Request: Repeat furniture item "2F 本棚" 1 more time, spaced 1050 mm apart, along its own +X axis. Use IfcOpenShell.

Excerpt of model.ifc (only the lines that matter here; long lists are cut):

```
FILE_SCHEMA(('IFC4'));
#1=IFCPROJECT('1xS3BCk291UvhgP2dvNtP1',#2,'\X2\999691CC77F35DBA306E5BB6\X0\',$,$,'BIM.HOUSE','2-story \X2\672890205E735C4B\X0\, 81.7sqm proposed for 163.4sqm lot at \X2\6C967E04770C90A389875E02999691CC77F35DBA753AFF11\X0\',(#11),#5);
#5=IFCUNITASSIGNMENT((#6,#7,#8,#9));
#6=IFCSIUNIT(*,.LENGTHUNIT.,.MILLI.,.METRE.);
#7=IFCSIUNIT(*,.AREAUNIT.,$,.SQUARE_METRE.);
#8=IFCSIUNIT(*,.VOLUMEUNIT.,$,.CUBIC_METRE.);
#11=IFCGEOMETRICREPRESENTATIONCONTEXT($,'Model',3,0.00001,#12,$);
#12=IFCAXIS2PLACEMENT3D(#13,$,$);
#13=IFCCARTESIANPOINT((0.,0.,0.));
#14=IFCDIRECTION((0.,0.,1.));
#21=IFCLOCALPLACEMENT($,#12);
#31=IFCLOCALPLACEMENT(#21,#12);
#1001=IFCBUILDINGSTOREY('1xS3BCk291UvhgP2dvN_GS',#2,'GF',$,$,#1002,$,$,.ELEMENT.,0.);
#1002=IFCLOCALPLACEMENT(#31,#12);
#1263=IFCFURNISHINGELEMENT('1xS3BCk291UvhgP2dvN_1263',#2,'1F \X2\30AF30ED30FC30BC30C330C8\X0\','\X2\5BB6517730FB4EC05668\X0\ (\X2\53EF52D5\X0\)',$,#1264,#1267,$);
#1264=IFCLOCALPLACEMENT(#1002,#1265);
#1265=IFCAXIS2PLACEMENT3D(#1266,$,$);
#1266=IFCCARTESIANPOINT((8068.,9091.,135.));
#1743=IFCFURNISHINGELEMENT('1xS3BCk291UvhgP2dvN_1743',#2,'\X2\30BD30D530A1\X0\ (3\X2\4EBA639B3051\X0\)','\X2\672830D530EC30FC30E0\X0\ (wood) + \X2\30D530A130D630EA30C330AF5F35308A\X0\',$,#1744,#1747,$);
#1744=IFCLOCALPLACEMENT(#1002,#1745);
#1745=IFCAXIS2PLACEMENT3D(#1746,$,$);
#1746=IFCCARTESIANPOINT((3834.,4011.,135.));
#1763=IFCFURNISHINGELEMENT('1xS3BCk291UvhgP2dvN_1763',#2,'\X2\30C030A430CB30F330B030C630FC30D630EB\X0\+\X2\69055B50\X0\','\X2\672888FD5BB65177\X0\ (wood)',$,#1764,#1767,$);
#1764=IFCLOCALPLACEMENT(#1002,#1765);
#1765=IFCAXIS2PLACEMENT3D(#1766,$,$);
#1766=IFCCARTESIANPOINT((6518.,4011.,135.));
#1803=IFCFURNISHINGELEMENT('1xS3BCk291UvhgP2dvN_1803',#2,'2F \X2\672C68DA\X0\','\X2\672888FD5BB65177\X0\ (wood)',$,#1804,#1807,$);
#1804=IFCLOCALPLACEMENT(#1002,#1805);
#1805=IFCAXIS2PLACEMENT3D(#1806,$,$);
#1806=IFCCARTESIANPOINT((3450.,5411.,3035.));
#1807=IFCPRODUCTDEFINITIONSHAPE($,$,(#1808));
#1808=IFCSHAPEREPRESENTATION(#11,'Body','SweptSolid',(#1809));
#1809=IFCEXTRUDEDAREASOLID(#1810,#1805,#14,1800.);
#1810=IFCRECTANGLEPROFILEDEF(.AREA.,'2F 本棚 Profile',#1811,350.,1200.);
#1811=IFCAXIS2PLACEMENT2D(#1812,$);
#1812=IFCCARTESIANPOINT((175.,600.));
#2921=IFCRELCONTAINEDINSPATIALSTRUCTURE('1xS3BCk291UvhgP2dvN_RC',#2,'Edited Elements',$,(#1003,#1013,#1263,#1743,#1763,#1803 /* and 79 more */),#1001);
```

```python
import ifcopenshell
import ifcopenshell.api.geometry
import ifcopenshell.api.root
import ifcopenshell.util.element
import ifcopenshell.util.placement

model = ifcopenshell.open("model.ifc")


def reuse_history(source, copy):
    """copy_class also copies each property set's owner history, people and application; keep the originals."""
    for rel in copy.IsDefinedBy:
        if rel.is_a("IfcRelDefinesByProperties") and (history := rel.RelatingPropertyDefinition.OwnerHistory):
            rel.RelatingPropertyDefinition.OwnerHistory = source.OwnerHistory
            ifcopenshell.util.element.remove_deep2(model, history)


source = model.by_guid("1xS3BCk291UvhgP2dvN_1803")
base = ifcopenshell.util.placement.get_local_placement(source.ObjectPlacement)
step = base[:3, 0] * 1050.0

for i in range(1, 2):
    copy = ifcopenshell.api.root.copy_class(model, product=source)
    copy.Representation = ifcopenshell.util.element.copy_deep(
        model, source.Representation, exclude=["IfcGeometricRepresentationContext", "IfcRepresentationMap"]
    )
    reuse_history(source, copy)
    matrix = base.copy()
    matrix[:3, 3] += i * step
    print("added at", matrix[:3, 3].round(3) + 0.0)
    ifcopenshell.api.geometry.edit_object_placement(model, product=copy, matrix=matrix, is_si=False)

model.write("model-out.ifc")
```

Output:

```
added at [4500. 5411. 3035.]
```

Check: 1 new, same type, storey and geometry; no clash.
